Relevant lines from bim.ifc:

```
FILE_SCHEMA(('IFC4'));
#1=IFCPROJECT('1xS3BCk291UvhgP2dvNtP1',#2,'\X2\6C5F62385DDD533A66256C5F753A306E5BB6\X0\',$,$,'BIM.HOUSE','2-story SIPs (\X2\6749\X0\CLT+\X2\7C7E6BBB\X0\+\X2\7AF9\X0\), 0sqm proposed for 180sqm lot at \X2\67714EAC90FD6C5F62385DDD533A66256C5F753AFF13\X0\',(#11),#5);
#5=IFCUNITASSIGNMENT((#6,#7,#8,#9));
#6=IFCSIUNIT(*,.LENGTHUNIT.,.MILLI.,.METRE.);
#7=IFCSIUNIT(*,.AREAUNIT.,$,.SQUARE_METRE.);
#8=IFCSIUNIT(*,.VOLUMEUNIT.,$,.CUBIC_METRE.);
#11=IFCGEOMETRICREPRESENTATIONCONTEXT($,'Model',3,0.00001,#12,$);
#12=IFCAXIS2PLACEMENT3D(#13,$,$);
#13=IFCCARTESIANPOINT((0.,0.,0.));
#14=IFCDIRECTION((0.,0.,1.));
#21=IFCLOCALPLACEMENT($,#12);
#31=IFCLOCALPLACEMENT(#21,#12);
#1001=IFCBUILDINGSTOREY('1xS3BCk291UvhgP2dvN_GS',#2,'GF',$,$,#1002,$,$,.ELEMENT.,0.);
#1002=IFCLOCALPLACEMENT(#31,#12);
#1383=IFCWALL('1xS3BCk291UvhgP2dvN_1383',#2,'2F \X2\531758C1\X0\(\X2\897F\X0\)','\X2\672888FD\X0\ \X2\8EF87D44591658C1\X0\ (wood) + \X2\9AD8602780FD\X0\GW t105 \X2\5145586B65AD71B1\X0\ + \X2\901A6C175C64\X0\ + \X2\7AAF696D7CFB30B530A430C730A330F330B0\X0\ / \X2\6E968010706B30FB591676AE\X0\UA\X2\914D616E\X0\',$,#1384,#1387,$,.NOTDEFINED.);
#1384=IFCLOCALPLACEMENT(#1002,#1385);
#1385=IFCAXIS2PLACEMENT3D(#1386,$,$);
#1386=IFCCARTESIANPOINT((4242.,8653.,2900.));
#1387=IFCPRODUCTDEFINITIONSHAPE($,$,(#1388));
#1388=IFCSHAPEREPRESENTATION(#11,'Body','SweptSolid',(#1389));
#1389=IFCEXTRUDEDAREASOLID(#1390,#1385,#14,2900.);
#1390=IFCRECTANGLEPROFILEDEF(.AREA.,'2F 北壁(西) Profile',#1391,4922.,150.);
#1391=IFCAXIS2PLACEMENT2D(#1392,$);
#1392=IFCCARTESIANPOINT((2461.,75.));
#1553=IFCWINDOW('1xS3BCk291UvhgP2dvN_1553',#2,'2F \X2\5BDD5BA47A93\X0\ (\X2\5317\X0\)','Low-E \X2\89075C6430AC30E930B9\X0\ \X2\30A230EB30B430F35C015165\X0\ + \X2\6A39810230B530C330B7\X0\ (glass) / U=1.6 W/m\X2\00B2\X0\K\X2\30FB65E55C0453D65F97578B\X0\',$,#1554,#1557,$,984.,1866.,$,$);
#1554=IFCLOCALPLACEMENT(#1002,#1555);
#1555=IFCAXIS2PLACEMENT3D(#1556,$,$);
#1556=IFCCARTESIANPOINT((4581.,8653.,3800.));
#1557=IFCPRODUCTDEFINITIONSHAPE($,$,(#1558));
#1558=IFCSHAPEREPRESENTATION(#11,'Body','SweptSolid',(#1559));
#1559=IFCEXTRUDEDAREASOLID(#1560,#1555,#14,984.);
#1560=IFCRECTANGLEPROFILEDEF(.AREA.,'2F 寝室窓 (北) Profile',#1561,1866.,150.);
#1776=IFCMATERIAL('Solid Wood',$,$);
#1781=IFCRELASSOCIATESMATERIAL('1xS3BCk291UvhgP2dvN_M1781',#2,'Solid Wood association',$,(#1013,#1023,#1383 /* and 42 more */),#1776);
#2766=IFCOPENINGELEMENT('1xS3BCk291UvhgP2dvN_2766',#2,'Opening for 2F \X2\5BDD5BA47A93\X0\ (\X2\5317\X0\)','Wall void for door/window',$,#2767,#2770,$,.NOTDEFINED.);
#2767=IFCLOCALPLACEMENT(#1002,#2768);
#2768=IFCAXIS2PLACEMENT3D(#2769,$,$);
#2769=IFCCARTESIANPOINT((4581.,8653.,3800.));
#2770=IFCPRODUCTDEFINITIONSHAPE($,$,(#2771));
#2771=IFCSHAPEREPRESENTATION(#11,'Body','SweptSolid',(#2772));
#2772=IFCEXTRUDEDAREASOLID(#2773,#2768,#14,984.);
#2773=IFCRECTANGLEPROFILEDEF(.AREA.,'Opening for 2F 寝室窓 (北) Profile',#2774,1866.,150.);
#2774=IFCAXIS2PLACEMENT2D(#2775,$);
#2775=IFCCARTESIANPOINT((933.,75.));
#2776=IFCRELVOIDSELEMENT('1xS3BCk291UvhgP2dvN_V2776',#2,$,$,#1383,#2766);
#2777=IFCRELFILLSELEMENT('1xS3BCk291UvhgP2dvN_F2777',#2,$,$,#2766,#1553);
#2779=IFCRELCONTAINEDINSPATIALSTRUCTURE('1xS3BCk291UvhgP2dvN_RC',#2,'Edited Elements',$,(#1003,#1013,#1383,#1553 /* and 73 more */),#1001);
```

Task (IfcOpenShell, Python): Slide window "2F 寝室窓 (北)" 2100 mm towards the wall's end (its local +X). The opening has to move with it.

```python
import ifcopenshell
import ifcopenshell.api.geometry
import ifcopenshell.util.placement

model = ifcopenshell.open("bim.ifc")

window = model.by_guid("1xS3BCk291UvhgP2dvN_1553")
opening = window.FillsVoids[0].RelatingOpeningElement
wall = opening.VoidsElements[0].RelatingBuildingElement

wall_matrix = ifcopenshell.util.placement.get_local_placement(wall.ObjectPlacement)
shift = wall_matrix[:3, 0] * 2100.0
before = ifcopenshell.util.placement.get_local_placement(window.ObjectPlacement)[:3, 3].copy()

# The window is not placed relative to its opening, so move both.
for product in (opening, window):
    matrix = ifcopenshell.util.placement.get_local_placement(product.ObjectPlacement)
    matrix[:3, 3] += shift
    ifcopenshell.api.geometry.edit_object_placement(model, product=product, matrix=matrix, is_si=False)

after = ifcopenshell.util.placement.get_local_placement(window.ObjectPlacement)[:3, 3]
print("window moved by", (after - before).round(3) + 0.0)

model.write("bim_edited.ifc")
```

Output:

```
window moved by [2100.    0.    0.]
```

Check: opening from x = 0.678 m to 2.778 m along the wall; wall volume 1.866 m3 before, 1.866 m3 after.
